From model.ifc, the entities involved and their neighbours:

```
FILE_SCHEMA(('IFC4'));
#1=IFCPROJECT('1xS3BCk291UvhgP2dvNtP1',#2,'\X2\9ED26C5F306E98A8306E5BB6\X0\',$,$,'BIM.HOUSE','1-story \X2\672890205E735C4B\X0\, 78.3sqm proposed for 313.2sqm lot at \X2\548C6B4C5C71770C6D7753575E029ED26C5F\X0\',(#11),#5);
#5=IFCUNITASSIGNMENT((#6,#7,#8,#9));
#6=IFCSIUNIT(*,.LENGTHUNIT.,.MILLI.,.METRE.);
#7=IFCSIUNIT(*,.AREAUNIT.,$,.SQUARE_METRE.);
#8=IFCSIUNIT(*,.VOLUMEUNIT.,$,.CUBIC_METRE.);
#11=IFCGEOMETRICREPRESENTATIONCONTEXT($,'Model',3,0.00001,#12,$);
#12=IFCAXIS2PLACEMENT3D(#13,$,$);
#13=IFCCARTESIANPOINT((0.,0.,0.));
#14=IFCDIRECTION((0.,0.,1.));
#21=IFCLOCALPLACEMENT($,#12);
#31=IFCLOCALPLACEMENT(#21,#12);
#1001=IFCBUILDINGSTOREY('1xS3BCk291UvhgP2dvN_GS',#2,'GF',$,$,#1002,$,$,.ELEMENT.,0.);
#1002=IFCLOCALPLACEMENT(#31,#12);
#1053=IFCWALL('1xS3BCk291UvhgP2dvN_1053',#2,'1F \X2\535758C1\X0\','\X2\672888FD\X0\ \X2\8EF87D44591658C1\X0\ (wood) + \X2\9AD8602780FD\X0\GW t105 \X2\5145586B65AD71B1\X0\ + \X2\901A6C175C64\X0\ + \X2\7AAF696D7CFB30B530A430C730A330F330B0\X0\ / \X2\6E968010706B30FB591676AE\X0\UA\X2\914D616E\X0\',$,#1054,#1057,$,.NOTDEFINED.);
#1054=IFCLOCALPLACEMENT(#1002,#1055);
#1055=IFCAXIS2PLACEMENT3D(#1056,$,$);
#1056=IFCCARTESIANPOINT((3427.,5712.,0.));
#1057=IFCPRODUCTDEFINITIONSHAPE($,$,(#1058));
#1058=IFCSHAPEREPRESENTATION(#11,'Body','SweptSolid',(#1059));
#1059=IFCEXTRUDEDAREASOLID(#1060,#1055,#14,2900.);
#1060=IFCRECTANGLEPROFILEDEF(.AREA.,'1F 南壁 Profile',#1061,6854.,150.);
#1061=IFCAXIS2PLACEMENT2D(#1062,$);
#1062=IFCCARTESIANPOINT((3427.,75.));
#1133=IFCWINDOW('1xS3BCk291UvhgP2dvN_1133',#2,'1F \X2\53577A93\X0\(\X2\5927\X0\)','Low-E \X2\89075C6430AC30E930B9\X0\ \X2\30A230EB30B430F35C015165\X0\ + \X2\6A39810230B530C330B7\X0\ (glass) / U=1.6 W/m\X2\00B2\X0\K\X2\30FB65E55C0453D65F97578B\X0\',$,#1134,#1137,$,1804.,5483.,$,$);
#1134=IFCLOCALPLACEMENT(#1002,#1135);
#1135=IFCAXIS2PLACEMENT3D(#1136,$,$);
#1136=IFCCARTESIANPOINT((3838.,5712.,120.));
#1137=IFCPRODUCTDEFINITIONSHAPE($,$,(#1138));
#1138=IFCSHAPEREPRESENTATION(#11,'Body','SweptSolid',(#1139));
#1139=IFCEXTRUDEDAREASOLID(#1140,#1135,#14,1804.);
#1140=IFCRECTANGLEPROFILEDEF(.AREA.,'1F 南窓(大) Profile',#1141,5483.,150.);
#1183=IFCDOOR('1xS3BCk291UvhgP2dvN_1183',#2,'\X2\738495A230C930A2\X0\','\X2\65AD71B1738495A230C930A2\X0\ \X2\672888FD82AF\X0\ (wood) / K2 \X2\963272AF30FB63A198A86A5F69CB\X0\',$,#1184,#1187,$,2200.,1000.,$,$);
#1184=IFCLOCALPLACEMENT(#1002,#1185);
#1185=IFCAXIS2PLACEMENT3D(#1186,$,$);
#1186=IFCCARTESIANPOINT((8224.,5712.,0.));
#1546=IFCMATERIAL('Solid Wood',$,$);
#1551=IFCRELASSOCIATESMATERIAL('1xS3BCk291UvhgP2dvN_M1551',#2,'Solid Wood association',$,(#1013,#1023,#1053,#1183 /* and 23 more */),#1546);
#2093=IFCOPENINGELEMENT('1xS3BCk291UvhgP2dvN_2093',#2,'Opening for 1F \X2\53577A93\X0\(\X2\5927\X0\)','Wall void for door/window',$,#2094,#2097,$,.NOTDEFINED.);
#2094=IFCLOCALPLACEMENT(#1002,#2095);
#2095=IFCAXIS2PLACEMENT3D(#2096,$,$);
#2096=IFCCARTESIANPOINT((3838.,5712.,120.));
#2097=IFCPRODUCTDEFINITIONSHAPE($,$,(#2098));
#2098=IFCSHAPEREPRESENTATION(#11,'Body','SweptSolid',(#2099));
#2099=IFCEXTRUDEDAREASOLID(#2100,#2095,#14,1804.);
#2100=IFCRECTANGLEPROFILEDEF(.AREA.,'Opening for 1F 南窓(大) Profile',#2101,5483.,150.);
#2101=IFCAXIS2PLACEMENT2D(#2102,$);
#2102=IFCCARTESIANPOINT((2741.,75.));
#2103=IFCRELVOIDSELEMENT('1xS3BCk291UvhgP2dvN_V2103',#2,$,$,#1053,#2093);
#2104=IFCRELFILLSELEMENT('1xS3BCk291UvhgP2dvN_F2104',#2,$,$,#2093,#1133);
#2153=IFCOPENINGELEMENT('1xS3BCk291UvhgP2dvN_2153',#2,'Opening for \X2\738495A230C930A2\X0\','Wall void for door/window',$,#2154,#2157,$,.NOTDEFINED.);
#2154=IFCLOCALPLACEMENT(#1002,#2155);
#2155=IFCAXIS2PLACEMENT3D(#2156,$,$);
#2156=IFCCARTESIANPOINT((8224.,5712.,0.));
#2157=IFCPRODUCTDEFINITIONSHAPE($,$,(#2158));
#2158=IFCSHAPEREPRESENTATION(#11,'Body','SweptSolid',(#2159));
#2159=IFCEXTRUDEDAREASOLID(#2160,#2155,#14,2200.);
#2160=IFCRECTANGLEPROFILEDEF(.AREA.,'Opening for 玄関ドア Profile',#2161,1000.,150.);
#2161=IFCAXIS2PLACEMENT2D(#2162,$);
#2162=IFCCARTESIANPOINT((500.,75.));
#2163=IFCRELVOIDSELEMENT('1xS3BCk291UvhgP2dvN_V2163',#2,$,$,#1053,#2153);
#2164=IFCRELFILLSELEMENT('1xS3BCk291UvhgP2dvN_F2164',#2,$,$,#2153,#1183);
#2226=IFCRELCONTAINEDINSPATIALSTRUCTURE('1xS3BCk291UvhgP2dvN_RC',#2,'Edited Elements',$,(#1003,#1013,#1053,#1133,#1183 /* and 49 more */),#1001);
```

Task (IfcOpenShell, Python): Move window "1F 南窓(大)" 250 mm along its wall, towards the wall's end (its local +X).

```python
import ifcopenshell
import ifcopenshell.api.geometry
import ifcopenshell.util.placement

model = ifcopenshell.open("model.ifc")

window = model.by_id(1133)
opening = window.FillsVoids[0].RelatingOpeningElement
wall = opening.VoidsElements[0].RelatingBuildingElement

wall_matrix = ifcopenshell.util.placement.get_local_placement(wall.ObjectPlacement)
shift = wall_matrix[:3, 0] * 250.0
before = ifcopenshell.util.placement.get_local_placement(window.ObjectPlacement)[:3, 3].copy()

# The window is not placed relative to its opening, so move both.
for product in (opening, window):
    matrix = ifcopenshell.util.placement.get_local_placement(product.ObjectPlacement)
    matrix[:3, 3] += shift
    ifcopenshell.api.geometry.edit_object_placement(model, product=product, matrix=matrix, is_si=False)

after = ifcopenshell.util.placement.get_local_placement(window.ObjectPlacement)[:3, 3]
print("window moved by", (after - before).round(3) + 0.0)

model.write("model_edited.ifc")
```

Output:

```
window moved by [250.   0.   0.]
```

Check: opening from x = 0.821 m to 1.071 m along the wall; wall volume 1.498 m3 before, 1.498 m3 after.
